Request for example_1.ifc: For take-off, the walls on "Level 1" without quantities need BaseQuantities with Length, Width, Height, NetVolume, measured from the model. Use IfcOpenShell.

First a look at what the model holds.

```python
import ifcopenshell
import ifcopenshell.util.element
import ifcopenshell.util.unit

model = ifcopenshell.open("example_1.ifc")
print(model.schema)
for unit_type in ("LENGTHUNIT", "AREAUNIT", "VOLUMEUNIT"):
    print(unit_type, ifcopenshell.util.unit.calculate_unit_scale(model, unit_type))
storey = next(s for s in model.by_type("IfcBuildingStorey") if s.Name == "Level 1")
walls = [e for e in ifcopenshell.util.element.get_decomposition(storey) if e.is_a("IfcWall")]
for e in sorted(walls, key=lambda e: e.id()):
    print(e.id(), e.is_a(), e.Name, list(ifcopenshell.util.element.get_psets(e, qtos_only=True)), sep=" | ")
```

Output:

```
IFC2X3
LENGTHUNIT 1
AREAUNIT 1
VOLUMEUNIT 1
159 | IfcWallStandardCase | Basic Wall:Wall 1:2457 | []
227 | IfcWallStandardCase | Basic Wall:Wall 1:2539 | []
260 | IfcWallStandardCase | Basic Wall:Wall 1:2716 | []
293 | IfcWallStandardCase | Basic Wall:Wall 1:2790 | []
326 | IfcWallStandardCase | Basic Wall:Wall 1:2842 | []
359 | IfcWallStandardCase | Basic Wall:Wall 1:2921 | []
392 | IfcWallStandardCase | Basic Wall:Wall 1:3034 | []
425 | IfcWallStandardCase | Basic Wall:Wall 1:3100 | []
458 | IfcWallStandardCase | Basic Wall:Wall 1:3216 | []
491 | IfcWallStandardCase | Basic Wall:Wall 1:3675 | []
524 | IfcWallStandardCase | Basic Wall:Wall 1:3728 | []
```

```python
import ifcopenshell
import ifcopenshell.api.pset
import ifcopenshell.geom
import ifcopenshell.util.element
import ifcopenshell.util.shape
import ifcopenshell.util.unit

model = ifcopenshell.open("example_1.ifc")
unit_scale = ifcopenshell.util.unit.calculate_unit_scale(model)
volume_scale = ifcopenshell.util.unit.calculate_unit_scale(model, "VOLUMEUNIT")
settings = ifcopenshell.geom.settings()

storey = next(s for s in model.by_type("IfcBuildingStorey") if s.Name == "Level 1")
walls = [e for e in ifcopenshell.util.element.get_decomposition(storey) if e.is_a("IfcWall")]

for e in sorted(walls, key=lambda e: e.id()):
    if ifcopenshell.util.element.get_psets(e, qtos_only=True, should_inherit=False):
        continue
    # Geometry comes back in metres, in the element's own axes.
    shape = ifcopenshell.geom.create_shape(settings, e)
    values = {
        "Length": ifcopenshell.util.shape.get_x(shape.geometry) / unit_scale,
        "Width": ifcopenshell.util.shape.get_y(shape.geometry) / unit_scale,
        "Height": ifcopenshell.util.shape.get_z(shape.geometry) / unit_scale,
        "NetVolume": ifcopenshell.util.shape.get_volume(shape.geometry) / volume_scale,
    }
    qto = ifcopenshell.api.pset.add_qto(model, product=e, name="BaseQuantities")
    ifcopenshell.api.pset.edit_qto(model, qto=qto, properties=values)
    print(e.id(), {k: round(v, 3) for k, v in values.items()})

model.write("example_1-out.ifc")
```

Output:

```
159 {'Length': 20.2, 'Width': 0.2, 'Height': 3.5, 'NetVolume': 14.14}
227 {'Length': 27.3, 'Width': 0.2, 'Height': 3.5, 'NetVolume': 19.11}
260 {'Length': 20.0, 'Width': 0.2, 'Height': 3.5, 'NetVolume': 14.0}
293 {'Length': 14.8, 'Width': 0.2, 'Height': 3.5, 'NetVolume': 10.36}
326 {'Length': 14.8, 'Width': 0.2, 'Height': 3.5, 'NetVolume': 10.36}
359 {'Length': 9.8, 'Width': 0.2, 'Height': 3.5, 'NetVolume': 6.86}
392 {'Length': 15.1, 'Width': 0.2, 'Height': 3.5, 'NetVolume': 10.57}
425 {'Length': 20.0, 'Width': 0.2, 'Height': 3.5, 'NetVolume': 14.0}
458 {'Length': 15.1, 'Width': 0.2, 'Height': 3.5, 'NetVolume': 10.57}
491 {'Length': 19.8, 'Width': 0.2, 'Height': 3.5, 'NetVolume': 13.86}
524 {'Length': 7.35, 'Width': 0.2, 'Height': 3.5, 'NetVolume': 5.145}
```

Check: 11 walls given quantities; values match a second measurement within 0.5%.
